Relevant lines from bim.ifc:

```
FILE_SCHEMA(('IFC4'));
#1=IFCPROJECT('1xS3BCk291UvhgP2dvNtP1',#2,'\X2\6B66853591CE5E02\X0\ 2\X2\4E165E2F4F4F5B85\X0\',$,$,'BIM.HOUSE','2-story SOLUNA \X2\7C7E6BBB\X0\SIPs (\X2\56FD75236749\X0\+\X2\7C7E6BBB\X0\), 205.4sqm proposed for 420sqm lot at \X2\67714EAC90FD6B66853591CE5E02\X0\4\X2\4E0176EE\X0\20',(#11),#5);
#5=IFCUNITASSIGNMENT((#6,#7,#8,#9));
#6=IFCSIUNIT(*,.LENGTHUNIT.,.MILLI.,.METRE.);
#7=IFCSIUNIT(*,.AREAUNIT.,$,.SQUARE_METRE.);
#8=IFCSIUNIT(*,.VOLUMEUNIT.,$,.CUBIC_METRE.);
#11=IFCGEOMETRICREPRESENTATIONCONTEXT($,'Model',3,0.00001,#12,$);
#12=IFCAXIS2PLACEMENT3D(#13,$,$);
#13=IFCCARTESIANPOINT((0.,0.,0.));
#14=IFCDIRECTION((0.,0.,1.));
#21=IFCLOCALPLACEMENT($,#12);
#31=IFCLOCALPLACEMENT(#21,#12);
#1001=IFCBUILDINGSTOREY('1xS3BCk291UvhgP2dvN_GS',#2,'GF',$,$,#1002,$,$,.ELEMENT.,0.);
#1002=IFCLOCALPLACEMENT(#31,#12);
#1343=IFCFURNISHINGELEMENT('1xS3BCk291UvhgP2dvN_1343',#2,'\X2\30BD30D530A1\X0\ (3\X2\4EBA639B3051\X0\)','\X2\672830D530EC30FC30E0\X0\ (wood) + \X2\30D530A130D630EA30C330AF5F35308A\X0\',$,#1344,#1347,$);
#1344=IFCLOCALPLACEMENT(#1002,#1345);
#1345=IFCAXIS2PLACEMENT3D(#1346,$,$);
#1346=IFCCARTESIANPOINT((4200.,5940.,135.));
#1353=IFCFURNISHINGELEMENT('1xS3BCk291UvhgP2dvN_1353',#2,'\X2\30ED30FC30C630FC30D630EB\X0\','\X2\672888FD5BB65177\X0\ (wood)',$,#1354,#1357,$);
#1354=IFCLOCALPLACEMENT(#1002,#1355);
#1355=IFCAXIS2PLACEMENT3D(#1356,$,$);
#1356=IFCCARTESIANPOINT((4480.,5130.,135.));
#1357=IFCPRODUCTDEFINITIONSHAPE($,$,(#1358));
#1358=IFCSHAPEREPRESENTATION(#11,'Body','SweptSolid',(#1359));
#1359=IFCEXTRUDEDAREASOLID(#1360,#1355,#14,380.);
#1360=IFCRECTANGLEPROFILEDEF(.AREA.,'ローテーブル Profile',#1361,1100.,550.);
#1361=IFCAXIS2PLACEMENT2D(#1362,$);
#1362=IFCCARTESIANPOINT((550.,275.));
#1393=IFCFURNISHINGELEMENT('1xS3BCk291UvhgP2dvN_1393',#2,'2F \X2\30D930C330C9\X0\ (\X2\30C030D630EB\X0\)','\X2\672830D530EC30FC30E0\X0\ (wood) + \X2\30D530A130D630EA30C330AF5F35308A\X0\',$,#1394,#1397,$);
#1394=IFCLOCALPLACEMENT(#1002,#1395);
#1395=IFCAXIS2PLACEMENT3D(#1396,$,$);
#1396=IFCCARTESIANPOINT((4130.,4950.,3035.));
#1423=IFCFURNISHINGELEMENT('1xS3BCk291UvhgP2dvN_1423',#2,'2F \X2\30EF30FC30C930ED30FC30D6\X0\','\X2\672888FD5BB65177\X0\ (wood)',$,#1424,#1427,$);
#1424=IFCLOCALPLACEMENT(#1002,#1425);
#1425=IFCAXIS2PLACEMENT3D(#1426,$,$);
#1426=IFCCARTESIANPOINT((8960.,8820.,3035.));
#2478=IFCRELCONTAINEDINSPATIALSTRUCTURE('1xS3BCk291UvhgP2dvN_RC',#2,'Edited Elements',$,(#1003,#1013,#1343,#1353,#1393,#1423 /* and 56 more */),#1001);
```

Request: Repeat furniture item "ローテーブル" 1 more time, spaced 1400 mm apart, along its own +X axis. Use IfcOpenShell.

```python
import ifcopenshell
import ifcopenshell.api.geometry
import ifcopenshell.api.root
import ifcopenshell.util.element
import ifcopenshell.util.placement

model = ifcopenshell.open("bim.ifc")


def reuse_history(source, copy):
    """copy_class also copies each property set's owner history, people and application; keep the originals."""
    for rel in copy.IsDefinedBy:
        if rel.is_a("IfcRelDefinesByProperties") and (history := rel.RelatingPropertyDefinition.OwnerHistory):
            rel.RelatingPropertyDefinition.OwnerHistory = source.OwnerHistory
            ifcopenshell.util.element.remove_deep2(model, history)


source = model.by_guid("1xS3BCk291UvhgP2dvN_1353")
base = ifcopenshell.util.placement.get_local_placement(source.ObjectPlacement)
step = base[:3, 0] * 1400.0

for i in range(1, 2):
    copy = ifcopenshell.api.root.copy_class(model, product=source)
    copy.Representation = ifcopenshell.util.element.copy_deep(
        model, source.Representation, exclude=["IfcGeometricRepresentationContext", "IfcRepresentationMap"]
    )
    reuse_history(source, copy)
    matrix = base.copy()
    matrix[:3, 3] += i * step
    print("added at", matrix[:3, 3].round(3) + 0.0)
    ifcopenshell.api.geometry.edit_object_placement(model, product=copy, matrix=matrix, is_si=False)

model.write("bim_rev.ifc")
```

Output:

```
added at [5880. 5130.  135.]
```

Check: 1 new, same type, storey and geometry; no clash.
